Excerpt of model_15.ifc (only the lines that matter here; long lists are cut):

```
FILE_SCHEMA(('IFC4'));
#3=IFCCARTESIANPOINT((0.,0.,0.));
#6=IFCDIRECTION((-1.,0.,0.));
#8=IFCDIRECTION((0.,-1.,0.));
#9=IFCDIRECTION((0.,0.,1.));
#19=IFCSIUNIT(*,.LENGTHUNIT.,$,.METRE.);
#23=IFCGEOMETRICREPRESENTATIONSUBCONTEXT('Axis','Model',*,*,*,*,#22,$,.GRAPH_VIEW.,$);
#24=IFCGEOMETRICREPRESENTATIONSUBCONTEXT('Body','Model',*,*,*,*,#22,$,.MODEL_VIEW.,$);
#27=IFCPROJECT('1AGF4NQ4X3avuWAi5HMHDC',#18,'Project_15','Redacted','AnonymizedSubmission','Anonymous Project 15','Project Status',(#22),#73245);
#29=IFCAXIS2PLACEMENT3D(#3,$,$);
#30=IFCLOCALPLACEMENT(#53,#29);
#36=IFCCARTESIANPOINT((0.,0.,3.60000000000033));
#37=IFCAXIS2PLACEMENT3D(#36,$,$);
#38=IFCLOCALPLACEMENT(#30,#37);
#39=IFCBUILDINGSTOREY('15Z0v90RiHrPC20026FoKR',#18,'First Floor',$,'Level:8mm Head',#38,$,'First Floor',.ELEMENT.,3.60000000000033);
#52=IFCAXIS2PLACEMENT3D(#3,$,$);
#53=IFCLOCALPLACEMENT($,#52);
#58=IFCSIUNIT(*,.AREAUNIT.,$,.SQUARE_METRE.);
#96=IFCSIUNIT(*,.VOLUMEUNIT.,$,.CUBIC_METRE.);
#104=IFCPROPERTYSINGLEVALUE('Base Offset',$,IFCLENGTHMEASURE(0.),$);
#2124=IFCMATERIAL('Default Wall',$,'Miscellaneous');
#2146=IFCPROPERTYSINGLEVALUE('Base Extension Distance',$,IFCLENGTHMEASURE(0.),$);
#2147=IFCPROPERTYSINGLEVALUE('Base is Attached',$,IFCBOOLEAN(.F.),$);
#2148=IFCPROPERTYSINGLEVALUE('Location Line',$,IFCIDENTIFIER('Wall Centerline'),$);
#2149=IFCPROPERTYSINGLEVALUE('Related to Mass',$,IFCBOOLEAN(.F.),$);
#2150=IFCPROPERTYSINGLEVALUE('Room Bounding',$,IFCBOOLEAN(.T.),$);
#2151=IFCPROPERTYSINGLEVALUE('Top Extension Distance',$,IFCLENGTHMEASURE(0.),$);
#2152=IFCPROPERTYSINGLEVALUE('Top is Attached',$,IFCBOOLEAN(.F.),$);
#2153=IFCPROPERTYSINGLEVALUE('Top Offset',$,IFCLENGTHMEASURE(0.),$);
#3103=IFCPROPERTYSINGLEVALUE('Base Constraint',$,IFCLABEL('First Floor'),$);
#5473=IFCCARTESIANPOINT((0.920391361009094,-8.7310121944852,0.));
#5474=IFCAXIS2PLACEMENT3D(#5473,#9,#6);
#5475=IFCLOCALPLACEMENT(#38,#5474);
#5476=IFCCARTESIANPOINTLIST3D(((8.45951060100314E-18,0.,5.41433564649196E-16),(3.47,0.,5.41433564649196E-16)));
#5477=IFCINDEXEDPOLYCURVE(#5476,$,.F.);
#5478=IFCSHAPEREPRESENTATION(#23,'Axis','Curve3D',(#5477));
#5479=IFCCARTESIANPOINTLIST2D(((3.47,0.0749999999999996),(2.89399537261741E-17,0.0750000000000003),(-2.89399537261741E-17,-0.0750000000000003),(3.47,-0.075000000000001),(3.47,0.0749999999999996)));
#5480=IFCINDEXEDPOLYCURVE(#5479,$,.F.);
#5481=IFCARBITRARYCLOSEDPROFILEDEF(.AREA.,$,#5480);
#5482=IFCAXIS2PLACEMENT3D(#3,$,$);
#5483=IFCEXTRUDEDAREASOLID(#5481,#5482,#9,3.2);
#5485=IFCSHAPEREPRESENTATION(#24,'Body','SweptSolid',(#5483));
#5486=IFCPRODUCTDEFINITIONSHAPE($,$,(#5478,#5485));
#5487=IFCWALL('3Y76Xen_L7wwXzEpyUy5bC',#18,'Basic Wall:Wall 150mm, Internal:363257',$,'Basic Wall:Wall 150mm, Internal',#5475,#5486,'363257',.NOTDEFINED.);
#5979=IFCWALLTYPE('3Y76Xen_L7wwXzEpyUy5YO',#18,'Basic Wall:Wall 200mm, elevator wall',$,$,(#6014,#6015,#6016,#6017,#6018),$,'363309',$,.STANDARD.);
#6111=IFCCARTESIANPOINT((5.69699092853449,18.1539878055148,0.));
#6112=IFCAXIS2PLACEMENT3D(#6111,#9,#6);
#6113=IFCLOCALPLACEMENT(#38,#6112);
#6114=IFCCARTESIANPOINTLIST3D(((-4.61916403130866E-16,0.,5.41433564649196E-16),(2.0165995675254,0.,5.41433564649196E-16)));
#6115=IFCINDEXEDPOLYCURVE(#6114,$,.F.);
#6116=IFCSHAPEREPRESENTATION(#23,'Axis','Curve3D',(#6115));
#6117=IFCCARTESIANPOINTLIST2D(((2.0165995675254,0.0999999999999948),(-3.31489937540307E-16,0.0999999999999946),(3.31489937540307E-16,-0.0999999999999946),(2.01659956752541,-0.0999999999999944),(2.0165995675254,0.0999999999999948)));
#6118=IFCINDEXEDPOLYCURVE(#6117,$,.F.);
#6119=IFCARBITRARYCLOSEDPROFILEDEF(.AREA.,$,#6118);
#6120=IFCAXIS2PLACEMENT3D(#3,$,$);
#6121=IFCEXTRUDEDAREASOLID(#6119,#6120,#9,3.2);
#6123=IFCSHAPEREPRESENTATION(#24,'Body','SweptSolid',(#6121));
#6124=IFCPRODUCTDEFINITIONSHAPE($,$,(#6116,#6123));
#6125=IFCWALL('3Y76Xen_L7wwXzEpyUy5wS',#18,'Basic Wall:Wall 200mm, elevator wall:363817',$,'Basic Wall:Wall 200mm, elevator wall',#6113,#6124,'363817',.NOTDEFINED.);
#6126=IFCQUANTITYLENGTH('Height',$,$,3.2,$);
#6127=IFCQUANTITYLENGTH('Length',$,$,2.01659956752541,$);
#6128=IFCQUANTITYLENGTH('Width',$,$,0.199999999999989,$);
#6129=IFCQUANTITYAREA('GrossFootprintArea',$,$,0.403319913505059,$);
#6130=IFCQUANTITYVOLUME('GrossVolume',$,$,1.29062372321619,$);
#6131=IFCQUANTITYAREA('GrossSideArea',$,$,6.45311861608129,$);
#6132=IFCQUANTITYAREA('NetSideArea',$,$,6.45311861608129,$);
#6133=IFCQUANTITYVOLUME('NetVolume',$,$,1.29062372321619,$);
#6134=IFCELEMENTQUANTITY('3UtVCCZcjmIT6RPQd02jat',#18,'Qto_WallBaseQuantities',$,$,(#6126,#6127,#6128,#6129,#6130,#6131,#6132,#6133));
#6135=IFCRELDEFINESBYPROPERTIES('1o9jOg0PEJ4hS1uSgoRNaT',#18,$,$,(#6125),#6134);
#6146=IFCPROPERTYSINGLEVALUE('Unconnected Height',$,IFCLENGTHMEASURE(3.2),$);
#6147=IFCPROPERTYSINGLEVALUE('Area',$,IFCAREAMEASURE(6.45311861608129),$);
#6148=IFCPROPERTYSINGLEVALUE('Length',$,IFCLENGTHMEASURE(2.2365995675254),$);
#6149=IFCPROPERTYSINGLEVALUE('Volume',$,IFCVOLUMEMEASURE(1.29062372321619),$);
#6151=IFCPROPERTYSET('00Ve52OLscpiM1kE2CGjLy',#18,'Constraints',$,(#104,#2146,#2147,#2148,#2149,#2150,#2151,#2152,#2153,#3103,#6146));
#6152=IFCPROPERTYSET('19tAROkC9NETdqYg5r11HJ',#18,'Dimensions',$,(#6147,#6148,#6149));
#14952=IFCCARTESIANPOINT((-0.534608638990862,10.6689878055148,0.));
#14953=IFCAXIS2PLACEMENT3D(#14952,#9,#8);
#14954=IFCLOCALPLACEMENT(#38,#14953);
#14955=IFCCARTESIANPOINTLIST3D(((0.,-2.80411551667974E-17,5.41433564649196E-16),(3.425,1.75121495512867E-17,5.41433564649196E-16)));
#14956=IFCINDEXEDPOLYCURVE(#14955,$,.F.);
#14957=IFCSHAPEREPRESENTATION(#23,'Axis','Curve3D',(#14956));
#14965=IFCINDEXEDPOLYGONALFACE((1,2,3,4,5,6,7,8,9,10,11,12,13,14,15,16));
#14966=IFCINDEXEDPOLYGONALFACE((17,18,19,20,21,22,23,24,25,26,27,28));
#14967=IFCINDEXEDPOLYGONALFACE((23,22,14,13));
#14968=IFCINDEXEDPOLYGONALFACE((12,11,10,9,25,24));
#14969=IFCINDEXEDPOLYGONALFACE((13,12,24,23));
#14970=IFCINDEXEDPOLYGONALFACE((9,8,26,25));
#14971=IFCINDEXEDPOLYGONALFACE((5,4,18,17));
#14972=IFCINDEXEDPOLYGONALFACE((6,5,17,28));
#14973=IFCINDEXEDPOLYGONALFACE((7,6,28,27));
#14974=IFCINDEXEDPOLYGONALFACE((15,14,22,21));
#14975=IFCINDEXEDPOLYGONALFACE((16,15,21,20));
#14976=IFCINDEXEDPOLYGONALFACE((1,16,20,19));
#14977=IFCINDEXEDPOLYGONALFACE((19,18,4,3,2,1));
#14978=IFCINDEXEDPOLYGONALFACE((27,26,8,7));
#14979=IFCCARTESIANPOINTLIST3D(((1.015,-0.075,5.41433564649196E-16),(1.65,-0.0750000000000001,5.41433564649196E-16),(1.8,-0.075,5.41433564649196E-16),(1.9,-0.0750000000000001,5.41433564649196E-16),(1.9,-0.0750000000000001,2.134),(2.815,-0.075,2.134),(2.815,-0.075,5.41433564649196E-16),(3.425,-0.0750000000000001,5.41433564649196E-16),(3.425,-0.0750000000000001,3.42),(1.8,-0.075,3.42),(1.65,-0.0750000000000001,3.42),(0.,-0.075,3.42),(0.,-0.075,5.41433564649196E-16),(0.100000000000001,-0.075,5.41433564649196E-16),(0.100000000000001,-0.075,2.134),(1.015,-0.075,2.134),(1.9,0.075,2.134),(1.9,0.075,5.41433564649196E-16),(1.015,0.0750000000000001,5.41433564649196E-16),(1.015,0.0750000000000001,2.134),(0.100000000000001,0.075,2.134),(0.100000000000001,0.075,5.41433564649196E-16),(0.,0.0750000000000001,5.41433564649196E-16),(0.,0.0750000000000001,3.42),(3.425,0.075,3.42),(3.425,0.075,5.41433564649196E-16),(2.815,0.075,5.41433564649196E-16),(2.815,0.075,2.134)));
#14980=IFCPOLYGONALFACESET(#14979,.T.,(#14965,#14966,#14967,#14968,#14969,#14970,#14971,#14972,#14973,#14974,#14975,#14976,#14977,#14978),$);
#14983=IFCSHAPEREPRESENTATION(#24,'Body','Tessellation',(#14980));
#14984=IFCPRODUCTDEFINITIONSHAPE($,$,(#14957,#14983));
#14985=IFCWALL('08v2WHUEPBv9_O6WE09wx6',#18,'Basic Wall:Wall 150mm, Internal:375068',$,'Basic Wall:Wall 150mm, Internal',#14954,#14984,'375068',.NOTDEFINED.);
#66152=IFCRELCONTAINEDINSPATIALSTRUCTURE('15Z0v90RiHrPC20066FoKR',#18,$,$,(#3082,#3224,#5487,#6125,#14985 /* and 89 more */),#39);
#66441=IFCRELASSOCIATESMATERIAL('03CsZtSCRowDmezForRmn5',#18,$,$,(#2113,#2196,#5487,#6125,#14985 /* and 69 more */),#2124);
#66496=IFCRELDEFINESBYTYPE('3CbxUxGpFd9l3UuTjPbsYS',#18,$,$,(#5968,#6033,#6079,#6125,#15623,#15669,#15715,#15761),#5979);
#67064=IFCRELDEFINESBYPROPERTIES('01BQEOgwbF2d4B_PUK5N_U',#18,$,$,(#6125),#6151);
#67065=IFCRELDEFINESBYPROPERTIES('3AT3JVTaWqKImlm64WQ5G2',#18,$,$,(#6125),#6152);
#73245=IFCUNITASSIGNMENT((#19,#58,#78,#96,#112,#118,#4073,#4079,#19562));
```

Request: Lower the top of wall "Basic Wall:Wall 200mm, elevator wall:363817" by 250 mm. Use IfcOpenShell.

```python
import ifcopenshell
import ifcopenshell.api.pset
import ifcopenshell.geom
import ifcopenshell.util.element
import ifcopenshell.util.representation
import ifcopenshell.util.shape
import ifcopenshell.util.unit

model = ifcopenshell.open("model_15.ifc")
unit_scale = ifcopenshell.util.unit.calculate_unit_scale(model)
area_scale = ifcopenshell.util.unit.calculate_unit_scale(model, "AREAUNIT")
volume_scale = ifcopenshell.util.unit.calculate_unit_scale(model, "VOLUMEUNIT")
settings = ifcopenshell.geom.settings()


def volume(element):
    """Net volume in cubic metres, openings subtracted."""
    shape = ifcopenshell.geom.create_shape(settings, element)
    return ifcopenshell.util.shape.get_volume(shape.geometry)


wall = model.by_guid("3Y76Xen_L7wwXzEpyUy5wS")
before = volume(wall)

body = ifcopenshell.util.representation.get_representation(wall, "Model", "Body")
solid = body.Items[0]
old_height = solid.Depth
solid.Depth -= 0.25 / unit_scale
after = volume(wall)
thickness = 0.2  # wall thickness in metres

# Update the stored height, areas and volumes.
qto = model.by_id(ifcopenshell.util.element.get_pset(wall, "Qto_WallBaseQuantities", should_inherit=False)["id"])
ifcopenshell.api.pset.edit_qto(model, qto=qto, properties={
    "Height": solid.Depth,
    "GrossVolume": ifcopenshell.util.element.get_pset(wall, "Qto_WallBaseQuantities", "GrossVolume") * solid.Depth / old_height,
    "GrossSideArea": ifcopenshell.util.element.get_pset(wall, "Qto_WallBaseQuantities", "GrossSideArea") * solid.Depth / old_height,
    "NetSideArea": after / thickness / area_scale,
    "NetVolume": after / volume_scale,
})
pset = model.by_id(ifcopenshell.util.element.get_pset(wall, "Constraints", should_inherit=False)["id"])
ifcopenshell.api.pset.edit_pset(model, pset=pset, properties={
    "Unconnected Height": model.create_entity("IfcLengthMeasure", solid.Depth),
})
pset = model.by_id(ifcopenshell.util.element.get_pset(wall, "Dimensions", should_inherit=False)["id"])
ifcopenshell.api.pset.edit_pset(model, pset=pset, properties={
    "Area": model.create_entity("IfcAreaMeasure", after / thickness / area_scale),
    "Volume": model.create_entity("IfcVolumeMeasure", after / volume_scale),
})

print(f"height {old_height:g} -> {solid.Depth:g}, volume {before:.3f} -> {after:.3f} m3")

model.write("model_15_updated.ifc")
```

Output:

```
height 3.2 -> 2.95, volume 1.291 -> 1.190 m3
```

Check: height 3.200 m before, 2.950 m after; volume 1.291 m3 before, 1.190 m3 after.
